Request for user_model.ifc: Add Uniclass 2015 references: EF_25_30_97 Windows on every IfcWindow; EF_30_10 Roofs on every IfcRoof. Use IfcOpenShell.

First a look at what the model holds.

```python
import ifcopenshell

model = ifcopenshell.open("user_model.ifc")
print(model.schema)
print("classifications:", [c.Name for c in model.by_type("IfcClassification")])
for ifc_class in ("IfcDoor", "IfcRoof", "IfcStair", "IfcWall", "IfcWindow"):
    print(ifc_class, len(model.by_type(ifc_class)))
```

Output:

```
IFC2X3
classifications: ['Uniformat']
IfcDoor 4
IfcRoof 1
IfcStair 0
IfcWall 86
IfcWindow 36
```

```python
import ifcopenshell
import ifcopenshell.api.classification

model = ifcopenshell.open("user_model.ifc")

# IFC2X3 requires Source and Edition and has no link from the project to the system.
system = model.create_entity("IfcClassification", Source="NBS", Edition="2015", Name="Uniclass 2015")

codes = {
    "IfcWindow": ("EF_25_30_97", "Windows"),
    "IfcRoof": ("EF_30_10", "Roofs"),
}
for ifc_class, (code, name) in codes.items():
    products = model.by_type(ifc_class)
    ifcopenshell.api.classification.add_reference(
        model, products=products, classification=system, identification=code, name=name
    )
    print(code, len(products))

model.write("user_model_rev.ifc")
```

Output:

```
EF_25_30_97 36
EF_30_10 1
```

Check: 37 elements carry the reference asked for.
